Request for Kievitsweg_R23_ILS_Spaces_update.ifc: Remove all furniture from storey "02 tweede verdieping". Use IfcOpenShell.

First a look at what the model holds.

```python
import ifcopenshell
import ifcopenshell.util.element

model = ifcopenshell.open("Kievitsweg_R23_ILS_Spaces_update.ifc")
print(model.schema)
storey = next(s for s in model.by_type("IfcBuildingStorey") if s.Name == "02 tweede verdieping")
furniture = [e for e in ifcopenshell.util.element.get_decomposition(storey) if e.is_a("IfcFurnishingElement")]
seen = {}
for e in furniture:
    element_type = ifcopenshell.util.element.get_type(e)
    name = element_type.Name if element_type not in (None, e) else None
    seen[name] = seen.get(name, 0) + 1
for name, count in sorted(seen.items(), key=str):
    print(count, "x", name)
```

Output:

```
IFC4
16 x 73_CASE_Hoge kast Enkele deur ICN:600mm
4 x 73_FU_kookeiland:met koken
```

```python
import ifcopenshell
import ifcopenshell.api.root
import ifcopenshell.util.element

model = ifcopenshell.open("Kievitsweg_R23_ILS_Spaces_update.ifc")

storey = next(s for s in model.by_type("IfcBuildingStorey") if s.Name == "02 tweede verdieping")
furniture = [e for e in ifcopenshell.util.element.get_decomposition(storey) if e.is_a("IfcFurnishingElement")]

for e in furniture:
    ifcopenshell.api.root.remove_product(model, product=e)
print(len(furniture), "removed")

model.write("Kievitsweg_R23_ILS_Spaces_update_v2.ifc")
```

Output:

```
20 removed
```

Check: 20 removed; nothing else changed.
